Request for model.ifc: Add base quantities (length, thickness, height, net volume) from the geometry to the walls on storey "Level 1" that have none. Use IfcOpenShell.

First a look at what the model holds.

```python
import ifcopenshell
import ifcopenshell.util.element
import ifcopenshell.util.unit

model = ifcopenshell.open("model.ifc")
print(model.schema)
for unit_type in ("LENGTHUNIT", "AREAUNIT", "VOLUMEUNIT"):
    print(unit_type, ifcopenshell.util.unit.calculate_unit_scale(model, unit_type))
storey = next(s for s in model.by_type("IfcBuildingStorey") if s.Name == "Level 1")
walls = [e for e in ifcopenshell.util.element.get_decomposition(storey) if e.is_a("IfcWall")]
for e in sorted(walls, key=lambda e: e.id()):
    print(e.id(), e.is_a(), e.Name, list(ifcopenshell.util.element.get_psets(e, qtos_only=True)), sep=" | ")
```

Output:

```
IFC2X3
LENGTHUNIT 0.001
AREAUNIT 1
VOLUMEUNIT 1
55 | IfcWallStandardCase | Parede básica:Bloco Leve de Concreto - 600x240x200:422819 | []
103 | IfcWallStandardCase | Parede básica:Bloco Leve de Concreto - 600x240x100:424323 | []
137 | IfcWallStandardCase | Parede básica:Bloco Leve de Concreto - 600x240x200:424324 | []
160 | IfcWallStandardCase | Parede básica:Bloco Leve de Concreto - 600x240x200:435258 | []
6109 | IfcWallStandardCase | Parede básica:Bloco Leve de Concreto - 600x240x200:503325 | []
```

```python
import ifcopenshell
import ifcopenshell.api.pset
import ifcopenshell.geom
import ifcopenshell.util.element
import ifcopenshell.util.shape
import ifcopenshell.util.unit

model = ifcopenshell.open("model.ifc")
unit_scale = ifcopenshell.util.unit.calculate_unit_scale(model)
volume_scale = ifcopenshell.util.unit.calculate_unit_scale(model, "VOLUMEUNIT")
settings = ifcopenshell.geom.settings()

storey = next(s for s in model.by_type("IfcBuildingStorey") if s.Name == "Level 1")
walls = [e for e in ifcopenshell.util.element.get_decomposition(storey) if e.is_a("IfcWall")]

for e in sorted(walls, key=lambda e: e.id()):
    if ifcopenshell.util.element.get_psets(e, qtos_only=True, should_inherit=False):
        continue
    # Geometry comes back in metres, in the element's own axes.
    shape = ifcopenshell.geom.create_shape(settings, e)
    values = {
        "Length": ifcopenshell.util.shape.get_x(shape.geometry) / unit_scale,
        "Width": ifcopenshell.util.shape.get_y(shape.geometry) / unit_scale,
        "Height": ifcopenshell.util.shape.get_z(shape.geometry) / unit_scale,
        "NetVolume": ifcopenshell.util.shape.get_volume(shape.geometry) / volume_scale,
    }
    qto = ifcopenshell.api.pset.add_qto(model, product=e, name="BaseQuantities")
    ifcopenshell.api.pset.edit_qto(model, qto=qto, properties=values)
    print(e.id(), {k: round(v, 3) for k, v in values.items()})

model.write("model-out.ifc")
```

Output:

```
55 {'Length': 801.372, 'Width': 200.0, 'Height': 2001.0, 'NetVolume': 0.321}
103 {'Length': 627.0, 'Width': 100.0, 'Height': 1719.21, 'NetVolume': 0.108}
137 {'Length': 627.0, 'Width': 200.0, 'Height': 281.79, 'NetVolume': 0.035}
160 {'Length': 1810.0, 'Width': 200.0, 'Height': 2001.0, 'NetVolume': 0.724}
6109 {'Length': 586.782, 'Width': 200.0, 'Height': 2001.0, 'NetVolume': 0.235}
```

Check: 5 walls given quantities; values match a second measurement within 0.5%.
